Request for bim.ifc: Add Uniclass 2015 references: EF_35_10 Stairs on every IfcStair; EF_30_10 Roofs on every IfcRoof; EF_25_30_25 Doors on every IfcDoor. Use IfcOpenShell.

First a look at what the model holds.

```python
import ifcopenshell

model = ifcopenshell.open("bim.ifc")
print(model.schema)
print("classifications:", [c.Name for c in model.by_type("IfcClassification")])
for ifc_class in ("IfcDoor", "IfcRoof", "IfcStair", "IfcWall", "IfcWindow"):
    print(ifc_class, len(model.by_type(ifc_class)))
```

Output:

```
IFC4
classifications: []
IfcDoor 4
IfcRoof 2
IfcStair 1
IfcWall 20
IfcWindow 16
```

```python
import ifcopenshell
import ifcopenshell.api.classification

model = ifcopenshell.open("bim.ifc")

system = ifcopenshell.api.classification.add_classification(model, classification="Uniclass 2015")

codes = {
    "IfcStair": ("EF_35_10", "Stairs"),
    "IfcRoof": ("EF_30_10", "Roofs"),
    "IfcDoor": ("EF_25_30_25", "Doors"),
}
for ifc_class, (code, name) in codes.items():
    products = model.by_type(ifc_class)
    ifcopenshell.api.classification.add_reference(
        model, products=products, classification=system, identification=code, name=name
    )
    print(code, len(products))

model.write("bim_v2.ifc")
```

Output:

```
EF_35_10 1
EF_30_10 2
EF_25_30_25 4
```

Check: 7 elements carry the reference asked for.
